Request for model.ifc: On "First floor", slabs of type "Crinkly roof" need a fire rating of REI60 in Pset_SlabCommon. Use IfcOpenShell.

First a look at what the model holds.

```python
import ifcopenshell
import ifcopenshell.util.element

model = ifcopenshell.open("model.ifc")
print(model.schema)
storey = next(s for s in model.by_type("IfcBuildingStorey") if s.Name == "First floor")
slabs = [e for e in ifcopenshell.util.element.get_decomposition(storey) if e.is_a("IfcSlab")]
seen = {}
for e in slabs:
    element_type = ifcopenshell.util.element.get_type(e)
    key = (element_type.Name if element_type != e and element_type else None, ifcopenshell.util.element.get_pset(e, "Pset_SlabCommon", "FireRating"))
    seen[key] = seen.get(key, 0) + 1
for (name, value), count in sorted(seen.items(), key=str):
    print(count, "x", name, "|", value)
```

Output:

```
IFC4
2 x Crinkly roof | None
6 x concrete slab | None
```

```python
import ifcopenshell
import ifcopenshell.api.pset
import ifcopenshell.util.element

model = ifcopenshell.open("model.ifc")

storey = next(s for s in model.by_type("IfcBuildingStorey") if s.Name == "First floor")
slabs = [e for e in ifcopenshell.util.element.get_decomposition(storey) if e.is_a("IfcSlab")]

count = 0
for e in slabs:
    element_type = ifcopenshell.util.element.get_type(e)
    if element_type in (None, e) or element_type.Name != "Crinkly roof":
        continue
    # add_pset returns the element's existing set when there is one.
    pset = ifcopenshell.api.pset.add_pset(model, product=e, name="Pset_SlabCommon")
    ifcopenshell.api.pset.edit_pset(model, pset=pset, properties={"FireRating": "REI60"})
    count += 1

print(count, "slabs updated")

model.write("model_edited.ifc")
```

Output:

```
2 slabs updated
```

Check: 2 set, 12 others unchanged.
